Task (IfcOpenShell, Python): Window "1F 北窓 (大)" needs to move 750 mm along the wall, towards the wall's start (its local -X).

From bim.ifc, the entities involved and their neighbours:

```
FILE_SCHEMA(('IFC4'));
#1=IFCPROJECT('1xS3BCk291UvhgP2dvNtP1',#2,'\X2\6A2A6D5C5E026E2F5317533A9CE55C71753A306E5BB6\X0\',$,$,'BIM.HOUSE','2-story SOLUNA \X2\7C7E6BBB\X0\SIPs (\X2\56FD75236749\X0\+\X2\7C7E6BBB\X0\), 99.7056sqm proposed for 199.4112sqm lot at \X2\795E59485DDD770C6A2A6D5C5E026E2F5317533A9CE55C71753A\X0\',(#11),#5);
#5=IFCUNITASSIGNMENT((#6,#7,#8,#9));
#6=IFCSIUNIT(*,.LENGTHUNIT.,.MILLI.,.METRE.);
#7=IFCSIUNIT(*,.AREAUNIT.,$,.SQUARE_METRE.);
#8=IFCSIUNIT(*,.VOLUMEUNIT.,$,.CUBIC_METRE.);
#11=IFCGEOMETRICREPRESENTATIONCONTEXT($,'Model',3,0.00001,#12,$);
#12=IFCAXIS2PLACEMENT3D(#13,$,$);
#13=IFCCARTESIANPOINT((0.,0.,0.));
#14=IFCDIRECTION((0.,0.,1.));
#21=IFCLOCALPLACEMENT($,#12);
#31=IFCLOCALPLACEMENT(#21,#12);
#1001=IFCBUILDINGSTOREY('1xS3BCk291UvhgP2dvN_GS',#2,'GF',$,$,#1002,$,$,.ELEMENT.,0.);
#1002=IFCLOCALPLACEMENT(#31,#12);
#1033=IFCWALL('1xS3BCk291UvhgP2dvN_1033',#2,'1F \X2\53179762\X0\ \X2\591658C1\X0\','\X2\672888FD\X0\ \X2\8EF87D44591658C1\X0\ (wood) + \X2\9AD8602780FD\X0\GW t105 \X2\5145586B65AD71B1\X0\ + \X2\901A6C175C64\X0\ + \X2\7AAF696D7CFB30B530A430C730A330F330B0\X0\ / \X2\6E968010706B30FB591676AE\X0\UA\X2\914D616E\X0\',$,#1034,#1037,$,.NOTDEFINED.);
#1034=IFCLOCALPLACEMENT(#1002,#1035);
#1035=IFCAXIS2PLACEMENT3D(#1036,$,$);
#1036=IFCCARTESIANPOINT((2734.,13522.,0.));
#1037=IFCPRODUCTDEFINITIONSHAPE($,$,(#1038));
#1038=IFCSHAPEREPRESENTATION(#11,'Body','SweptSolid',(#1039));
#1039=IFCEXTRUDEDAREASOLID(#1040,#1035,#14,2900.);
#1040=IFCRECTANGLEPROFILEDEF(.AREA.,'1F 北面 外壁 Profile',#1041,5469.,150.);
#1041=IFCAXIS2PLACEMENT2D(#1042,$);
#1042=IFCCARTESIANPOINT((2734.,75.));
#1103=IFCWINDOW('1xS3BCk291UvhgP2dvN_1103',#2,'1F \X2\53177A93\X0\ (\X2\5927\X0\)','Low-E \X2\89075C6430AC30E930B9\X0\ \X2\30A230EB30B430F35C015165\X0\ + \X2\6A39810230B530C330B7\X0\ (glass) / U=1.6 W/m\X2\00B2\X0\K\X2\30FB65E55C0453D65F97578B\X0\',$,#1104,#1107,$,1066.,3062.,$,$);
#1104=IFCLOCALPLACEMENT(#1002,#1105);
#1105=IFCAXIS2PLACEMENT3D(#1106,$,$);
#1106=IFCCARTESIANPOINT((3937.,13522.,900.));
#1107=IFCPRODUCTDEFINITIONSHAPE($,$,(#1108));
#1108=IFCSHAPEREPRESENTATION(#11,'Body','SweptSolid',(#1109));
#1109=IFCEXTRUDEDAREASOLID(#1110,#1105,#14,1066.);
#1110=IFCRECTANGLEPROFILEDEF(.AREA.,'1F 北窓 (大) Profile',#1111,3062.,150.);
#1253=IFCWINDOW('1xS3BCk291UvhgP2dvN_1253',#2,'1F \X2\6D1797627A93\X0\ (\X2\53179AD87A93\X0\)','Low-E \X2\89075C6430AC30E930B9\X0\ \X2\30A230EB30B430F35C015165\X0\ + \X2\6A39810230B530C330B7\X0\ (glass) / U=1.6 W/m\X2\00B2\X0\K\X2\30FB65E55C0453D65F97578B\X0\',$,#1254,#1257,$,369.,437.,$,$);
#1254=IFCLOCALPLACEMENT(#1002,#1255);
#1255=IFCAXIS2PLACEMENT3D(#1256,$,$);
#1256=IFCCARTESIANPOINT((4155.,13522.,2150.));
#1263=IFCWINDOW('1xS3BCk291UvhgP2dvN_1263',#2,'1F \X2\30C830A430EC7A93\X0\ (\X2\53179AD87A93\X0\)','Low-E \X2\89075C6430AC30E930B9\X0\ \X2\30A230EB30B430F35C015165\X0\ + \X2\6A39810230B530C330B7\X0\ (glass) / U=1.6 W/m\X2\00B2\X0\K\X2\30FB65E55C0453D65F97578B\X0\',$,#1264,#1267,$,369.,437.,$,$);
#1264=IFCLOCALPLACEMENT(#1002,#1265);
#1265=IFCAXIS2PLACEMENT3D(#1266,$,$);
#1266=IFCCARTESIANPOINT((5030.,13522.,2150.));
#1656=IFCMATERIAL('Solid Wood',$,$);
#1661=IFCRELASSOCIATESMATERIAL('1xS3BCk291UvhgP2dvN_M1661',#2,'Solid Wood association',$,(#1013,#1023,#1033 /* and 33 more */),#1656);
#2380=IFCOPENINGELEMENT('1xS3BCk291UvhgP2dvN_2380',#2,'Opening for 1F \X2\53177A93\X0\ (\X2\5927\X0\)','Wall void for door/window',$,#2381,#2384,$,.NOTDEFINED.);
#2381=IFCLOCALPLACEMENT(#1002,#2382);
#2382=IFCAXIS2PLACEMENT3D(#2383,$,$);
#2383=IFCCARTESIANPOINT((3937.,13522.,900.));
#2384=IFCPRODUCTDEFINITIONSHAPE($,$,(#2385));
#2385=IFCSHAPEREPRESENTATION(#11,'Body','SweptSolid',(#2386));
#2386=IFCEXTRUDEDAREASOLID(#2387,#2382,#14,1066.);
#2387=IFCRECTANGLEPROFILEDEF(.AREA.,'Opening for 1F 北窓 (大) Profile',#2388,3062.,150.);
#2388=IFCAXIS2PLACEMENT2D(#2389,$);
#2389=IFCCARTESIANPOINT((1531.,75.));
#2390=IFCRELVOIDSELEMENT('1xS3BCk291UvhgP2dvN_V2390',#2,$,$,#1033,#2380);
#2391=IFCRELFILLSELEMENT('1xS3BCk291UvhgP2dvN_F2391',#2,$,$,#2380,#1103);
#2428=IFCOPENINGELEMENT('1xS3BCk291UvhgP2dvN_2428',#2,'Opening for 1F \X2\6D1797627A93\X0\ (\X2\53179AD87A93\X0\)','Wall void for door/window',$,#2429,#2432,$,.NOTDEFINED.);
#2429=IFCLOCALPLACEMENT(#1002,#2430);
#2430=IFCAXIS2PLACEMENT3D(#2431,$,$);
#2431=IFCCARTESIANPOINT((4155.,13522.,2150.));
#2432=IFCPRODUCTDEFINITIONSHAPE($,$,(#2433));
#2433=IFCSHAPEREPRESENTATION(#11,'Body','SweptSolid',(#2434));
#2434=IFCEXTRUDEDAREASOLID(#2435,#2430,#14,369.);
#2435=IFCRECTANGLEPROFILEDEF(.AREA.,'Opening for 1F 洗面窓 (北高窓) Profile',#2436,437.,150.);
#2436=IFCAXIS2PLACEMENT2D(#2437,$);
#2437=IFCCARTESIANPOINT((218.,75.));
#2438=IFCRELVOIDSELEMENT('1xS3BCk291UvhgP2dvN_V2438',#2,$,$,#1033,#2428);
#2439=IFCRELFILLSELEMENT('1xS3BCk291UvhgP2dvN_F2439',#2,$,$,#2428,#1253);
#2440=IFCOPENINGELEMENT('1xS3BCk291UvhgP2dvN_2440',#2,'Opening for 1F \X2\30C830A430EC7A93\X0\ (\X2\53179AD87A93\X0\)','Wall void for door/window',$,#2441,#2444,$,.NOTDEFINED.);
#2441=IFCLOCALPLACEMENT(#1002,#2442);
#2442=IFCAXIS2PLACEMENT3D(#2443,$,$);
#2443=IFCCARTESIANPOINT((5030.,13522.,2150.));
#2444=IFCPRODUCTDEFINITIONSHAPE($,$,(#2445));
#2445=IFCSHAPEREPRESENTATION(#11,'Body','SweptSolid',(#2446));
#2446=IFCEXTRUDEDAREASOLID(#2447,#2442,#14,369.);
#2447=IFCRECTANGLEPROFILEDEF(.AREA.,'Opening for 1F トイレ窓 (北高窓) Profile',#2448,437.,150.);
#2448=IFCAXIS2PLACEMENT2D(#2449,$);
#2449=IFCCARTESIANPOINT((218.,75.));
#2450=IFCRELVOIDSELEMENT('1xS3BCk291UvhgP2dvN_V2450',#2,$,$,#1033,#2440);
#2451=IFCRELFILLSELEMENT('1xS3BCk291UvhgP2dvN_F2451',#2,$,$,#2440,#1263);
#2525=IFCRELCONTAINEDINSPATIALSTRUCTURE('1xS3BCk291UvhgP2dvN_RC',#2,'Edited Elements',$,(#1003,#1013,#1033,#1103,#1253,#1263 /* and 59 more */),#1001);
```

```python
import ifcopenshell
import ifcopenshell.api.geometry
import ifcopenshell.util.placement
import ifcopenshell.util.unit

model = ifcopenshell.open("bim.ifc")
unit_scale = ifcopenshell.util.unit.calculate_unit_scale(model)

window = model.by_guid("1xS3BCk291UvhgP2dvN_1103")
opening = window.FillsVoids[0].RelatingOpeningElement
wall = opening.VoidsElements[0].RelatingBuildingElement

wall_matrix = ifcopenshell.util.placement.get_local_placement(wall.ObjectPlacement)
shift = wall_matrix[:3, 0] * -0.75 / unit_scale
before = ifcopenshell.util.placement.get_local_placement(window.ObjectPlacement)[:3, 3].copy()

# The window is not placed relative to its opening, so move both.
for product in (opening, window):
    matrix = ifcopenshell.util.placement.get_local_placement(product.ObjectPlacement)
    matrix[:3, 3] += shift
    ifcopenshell.api.geometry.edit_object_placement(model, product=product, matrix=matrix, is_si=False)

after = ifcopenshell.util.placement.get_local_placement(window.ObjectPlacement)[:3, 3]
print("window moved by", (after - before).round(3) + 0.0)

model.write("bim_v2.ifc")
```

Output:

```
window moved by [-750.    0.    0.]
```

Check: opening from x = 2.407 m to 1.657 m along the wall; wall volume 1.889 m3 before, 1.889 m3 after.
